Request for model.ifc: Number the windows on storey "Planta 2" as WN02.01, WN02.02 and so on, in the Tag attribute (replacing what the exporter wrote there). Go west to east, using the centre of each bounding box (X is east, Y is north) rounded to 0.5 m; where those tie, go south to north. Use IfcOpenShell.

First a look at what the model holds.

```python
import ifcopenshell
import ifcopenshell.util.element
import ifcopenshell.util.placement

model = ifcopenshell.open("model.ifc")
print(model.schema)
storey = next(s for s in model.by_type("IfcBuildingStorey") if s.Name == "Planta 2")
windows = [e for e in ifcopenshell.util.element.get_decomposition(storey) if e.is_a("IfcWindow")]
for e in sorted(windows, key=lambda e: e.id()):
    origin = ifcopenshell.util.placement.get_local_placement(e.ObjectPlacement)[:3, 3]
    print(e.id(), e.Tag, e.Name, origin.round(2) + 0.0, sep=" | ")
```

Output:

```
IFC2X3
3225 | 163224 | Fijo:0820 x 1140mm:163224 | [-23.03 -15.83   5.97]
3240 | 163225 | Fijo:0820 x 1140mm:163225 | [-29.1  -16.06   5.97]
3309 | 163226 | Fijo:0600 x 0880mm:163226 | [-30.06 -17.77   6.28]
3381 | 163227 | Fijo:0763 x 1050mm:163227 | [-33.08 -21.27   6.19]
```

```python
import ifcopenshell
import ifcopenshell.geom
import ifcopenshell.util.element
import ifcopenshell.util.shape

model = ifcopenshell.open("model.ifc")
settings = ifcopenshell.geom.settings()
settings.set("use-world-coords", True)


def centre(element):
    shape = ifcopenshell.geom.create_shape(settings, element)
    return ifcopenshell.util.shape.get_bbox_centroid(shape.geometry)


storey = next(s for s in model.by_type("IfcBuildingStorey") if s.Name == "Planta 2")
windows = [e for e in ifcopenshell.util.element.get_decomposition(storey) if e.is_a("IfcWindow")]

# Insertion points can sit at a corner or the storey origin, so sort by the geometry (in metres).
centres = {e: centre(e) for e in windows}
windows.sort(key=lambda e: (round(centres[e][0] / 0.5), centres[e][1]))

for i, e in enumerate(windows, start=1):
    number = f"WN02.{i:02d}"
    e.Tag = number
    print(e.id(), number)

model.write("model_updated.ifc")
```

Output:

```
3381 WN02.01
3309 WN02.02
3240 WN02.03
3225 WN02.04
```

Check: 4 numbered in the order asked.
